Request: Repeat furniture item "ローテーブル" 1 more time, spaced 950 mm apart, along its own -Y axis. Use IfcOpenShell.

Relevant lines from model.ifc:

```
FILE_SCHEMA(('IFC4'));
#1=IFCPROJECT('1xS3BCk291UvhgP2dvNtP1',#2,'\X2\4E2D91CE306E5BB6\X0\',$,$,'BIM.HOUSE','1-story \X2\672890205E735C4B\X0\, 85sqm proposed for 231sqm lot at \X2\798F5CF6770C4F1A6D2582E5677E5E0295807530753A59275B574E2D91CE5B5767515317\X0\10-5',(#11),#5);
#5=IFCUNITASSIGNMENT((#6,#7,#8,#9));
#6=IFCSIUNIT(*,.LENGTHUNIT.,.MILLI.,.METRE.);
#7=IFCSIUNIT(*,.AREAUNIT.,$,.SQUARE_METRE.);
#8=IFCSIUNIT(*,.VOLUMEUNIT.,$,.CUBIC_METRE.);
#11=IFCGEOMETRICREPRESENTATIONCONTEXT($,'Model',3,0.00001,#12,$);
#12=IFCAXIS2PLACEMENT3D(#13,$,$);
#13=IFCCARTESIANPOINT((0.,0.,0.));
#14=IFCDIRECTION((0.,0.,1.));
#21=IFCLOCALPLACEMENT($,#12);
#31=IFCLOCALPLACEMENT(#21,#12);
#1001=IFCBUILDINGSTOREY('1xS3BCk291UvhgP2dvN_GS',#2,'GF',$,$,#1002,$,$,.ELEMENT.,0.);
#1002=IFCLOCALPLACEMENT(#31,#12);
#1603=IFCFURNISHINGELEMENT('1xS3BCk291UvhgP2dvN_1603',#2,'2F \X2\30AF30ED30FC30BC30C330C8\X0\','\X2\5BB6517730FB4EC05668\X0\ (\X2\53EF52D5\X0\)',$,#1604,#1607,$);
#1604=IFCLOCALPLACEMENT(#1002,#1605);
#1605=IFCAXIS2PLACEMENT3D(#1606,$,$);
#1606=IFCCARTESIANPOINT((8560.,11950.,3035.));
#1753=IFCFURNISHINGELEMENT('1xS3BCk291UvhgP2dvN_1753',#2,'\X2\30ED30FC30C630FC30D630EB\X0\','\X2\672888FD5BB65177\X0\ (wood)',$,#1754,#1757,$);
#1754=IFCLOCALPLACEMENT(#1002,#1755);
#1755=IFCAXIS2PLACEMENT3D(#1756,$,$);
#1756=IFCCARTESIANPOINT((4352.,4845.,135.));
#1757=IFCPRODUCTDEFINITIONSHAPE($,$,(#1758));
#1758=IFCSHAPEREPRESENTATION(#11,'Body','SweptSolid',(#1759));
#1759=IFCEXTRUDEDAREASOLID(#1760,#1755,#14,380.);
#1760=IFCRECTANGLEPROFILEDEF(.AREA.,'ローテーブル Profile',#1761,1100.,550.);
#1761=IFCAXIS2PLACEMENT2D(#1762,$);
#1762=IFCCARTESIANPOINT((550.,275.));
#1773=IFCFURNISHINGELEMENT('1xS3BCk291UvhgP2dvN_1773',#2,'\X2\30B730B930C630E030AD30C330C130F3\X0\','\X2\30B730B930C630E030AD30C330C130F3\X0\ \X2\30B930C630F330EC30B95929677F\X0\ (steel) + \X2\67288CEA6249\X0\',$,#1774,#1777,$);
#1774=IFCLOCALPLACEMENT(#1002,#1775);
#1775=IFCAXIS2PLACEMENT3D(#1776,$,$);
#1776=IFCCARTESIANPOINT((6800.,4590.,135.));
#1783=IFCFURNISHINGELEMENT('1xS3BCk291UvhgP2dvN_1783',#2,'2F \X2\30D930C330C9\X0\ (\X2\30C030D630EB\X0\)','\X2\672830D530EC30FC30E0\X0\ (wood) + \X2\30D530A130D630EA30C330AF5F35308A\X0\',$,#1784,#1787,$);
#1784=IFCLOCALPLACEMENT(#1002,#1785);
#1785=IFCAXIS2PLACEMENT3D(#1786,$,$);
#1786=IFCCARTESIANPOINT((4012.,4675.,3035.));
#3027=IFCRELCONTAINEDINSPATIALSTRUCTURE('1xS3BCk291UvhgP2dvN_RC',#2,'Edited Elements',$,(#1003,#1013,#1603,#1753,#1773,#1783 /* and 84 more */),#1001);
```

```python
import ifcopenshell
import ifcopenshell.api.geometry
import ifcopenshell.api.root
import ifcopenshell.util.element
import ifcopenshell.util.placement

model = ifcopenshell.open("model.ifc")


def reuse_history(source, copy):
    """copy_class also copies each property set's owner history, people and application; keep the originals."""
    for rel in copy.IsDefinedBy:
        if rel.is_a("IfcRelDefinesByProperties") and (history := rel.RelatingPropertyDefinition.OwnerHistory):
            rel.RelatingPropertyDefinition.OwnerHistory = source.OwnerHistory
            ifcopenshell.util.element.remove_deep2(model, history)


source = model.by_id(1753)
base = ifcopenshell.util.placement.get_local_placement(source.ObjectPlacement)
step = -base[:3, 1] * 950.0

for i in range(1, 2):
    copy = ifcopenshell.api.root.copy_class(model, product=source)
    copy.Representation = ifcopenshell.util.element.copy_deep(
        model, source.Representation, exclude=["IfcGeometricRepresentationContext", "IfcRepresentationMap"]
    )
    reuse_history(source, copy)
    matrix = base.copy()
    matrix[:3, 3] += i * step
    print("added at", matrix[:3, 3].round(3) + 0.0)
    ifcopenshell.api.geometry.edit_object_placement(model, product=copy, matrix=matrix, is_si=False)

model.write("model-out.ifc")
```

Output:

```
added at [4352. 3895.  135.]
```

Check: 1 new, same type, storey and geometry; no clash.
